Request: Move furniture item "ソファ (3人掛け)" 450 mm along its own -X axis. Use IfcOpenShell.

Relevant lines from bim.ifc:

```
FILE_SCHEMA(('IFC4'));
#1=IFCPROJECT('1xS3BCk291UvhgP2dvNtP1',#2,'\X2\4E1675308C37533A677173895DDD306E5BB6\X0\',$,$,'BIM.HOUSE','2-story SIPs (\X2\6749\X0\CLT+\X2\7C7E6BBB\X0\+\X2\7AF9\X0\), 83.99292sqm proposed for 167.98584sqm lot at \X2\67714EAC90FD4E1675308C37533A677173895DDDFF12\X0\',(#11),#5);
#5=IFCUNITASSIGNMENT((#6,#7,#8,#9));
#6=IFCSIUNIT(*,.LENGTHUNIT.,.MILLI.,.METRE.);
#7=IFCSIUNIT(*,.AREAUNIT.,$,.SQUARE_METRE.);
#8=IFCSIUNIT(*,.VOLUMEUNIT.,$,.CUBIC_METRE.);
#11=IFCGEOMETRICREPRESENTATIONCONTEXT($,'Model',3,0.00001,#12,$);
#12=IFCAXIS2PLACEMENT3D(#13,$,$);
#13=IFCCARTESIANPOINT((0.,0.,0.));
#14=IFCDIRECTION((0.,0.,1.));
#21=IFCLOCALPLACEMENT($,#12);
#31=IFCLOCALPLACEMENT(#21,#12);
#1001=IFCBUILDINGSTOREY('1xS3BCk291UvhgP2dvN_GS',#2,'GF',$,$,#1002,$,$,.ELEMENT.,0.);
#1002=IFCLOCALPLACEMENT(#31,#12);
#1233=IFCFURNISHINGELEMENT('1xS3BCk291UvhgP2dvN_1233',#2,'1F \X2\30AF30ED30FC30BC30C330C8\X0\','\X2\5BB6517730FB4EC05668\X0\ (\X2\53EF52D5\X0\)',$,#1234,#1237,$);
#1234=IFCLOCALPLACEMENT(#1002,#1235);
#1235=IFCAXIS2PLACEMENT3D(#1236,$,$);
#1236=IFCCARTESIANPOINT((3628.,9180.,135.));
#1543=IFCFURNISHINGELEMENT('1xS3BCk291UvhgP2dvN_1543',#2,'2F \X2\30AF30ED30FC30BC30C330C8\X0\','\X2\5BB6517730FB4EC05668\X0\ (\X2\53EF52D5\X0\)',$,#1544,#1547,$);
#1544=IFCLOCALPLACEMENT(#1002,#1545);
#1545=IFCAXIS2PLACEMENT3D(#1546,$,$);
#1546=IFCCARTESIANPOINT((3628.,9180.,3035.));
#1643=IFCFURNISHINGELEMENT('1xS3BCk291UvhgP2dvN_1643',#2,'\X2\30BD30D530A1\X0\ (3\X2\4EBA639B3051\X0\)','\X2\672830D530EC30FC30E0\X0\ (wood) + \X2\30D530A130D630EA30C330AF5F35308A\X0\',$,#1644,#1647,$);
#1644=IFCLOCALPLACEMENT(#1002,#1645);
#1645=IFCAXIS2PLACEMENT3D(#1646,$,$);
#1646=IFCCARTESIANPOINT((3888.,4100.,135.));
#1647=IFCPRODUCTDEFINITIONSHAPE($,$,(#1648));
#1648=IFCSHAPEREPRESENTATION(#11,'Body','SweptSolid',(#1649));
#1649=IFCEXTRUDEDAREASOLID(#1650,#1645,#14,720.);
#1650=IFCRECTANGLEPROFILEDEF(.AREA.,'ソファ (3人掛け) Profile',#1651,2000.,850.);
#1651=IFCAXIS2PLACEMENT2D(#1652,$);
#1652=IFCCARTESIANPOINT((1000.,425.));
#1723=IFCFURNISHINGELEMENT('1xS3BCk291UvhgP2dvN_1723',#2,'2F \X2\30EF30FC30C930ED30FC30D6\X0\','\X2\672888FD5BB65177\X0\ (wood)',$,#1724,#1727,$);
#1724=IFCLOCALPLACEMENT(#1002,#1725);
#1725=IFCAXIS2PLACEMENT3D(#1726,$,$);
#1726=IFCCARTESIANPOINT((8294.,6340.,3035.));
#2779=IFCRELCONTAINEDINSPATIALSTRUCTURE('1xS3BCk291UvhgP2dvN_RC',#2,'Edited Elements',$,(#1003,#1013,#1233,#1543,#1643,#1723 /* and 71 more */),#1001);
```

```python
import ifcopenshell
import ifcopenshell.api.geometry
import ifcopenshell.util.placement
import ifcopenshell.util.unit

model = ifcopenshell.open("bim.ifc")
unit_scale = ifcopenshell.util.unit.calculate_unit_scale(model)

item = model.by_id(1643)
matrix = ifcopenshell.util.placement.get_local_placement(item.ObjectPlacement)
matrix[:3, 3] -= matrix[:3, 0] * 0.45 / unit_scale
ifcopenshell.api.geometry.edit_object_placement(model, product=item, matrix=matrix, is_si=False)

print(ifcopenshell.util.placement.get_local_placement(item.ObjectPlacement).round(3) + 0.0)

model.write("bim_edited.ifc")
```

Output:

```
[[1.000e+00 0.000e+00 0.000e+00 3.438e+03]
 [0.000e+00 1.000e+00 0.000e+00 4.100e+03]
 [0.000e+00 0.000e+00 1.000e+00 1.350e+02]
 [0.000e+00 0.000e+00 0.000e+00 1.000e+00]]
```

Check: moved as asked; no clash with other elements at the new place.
